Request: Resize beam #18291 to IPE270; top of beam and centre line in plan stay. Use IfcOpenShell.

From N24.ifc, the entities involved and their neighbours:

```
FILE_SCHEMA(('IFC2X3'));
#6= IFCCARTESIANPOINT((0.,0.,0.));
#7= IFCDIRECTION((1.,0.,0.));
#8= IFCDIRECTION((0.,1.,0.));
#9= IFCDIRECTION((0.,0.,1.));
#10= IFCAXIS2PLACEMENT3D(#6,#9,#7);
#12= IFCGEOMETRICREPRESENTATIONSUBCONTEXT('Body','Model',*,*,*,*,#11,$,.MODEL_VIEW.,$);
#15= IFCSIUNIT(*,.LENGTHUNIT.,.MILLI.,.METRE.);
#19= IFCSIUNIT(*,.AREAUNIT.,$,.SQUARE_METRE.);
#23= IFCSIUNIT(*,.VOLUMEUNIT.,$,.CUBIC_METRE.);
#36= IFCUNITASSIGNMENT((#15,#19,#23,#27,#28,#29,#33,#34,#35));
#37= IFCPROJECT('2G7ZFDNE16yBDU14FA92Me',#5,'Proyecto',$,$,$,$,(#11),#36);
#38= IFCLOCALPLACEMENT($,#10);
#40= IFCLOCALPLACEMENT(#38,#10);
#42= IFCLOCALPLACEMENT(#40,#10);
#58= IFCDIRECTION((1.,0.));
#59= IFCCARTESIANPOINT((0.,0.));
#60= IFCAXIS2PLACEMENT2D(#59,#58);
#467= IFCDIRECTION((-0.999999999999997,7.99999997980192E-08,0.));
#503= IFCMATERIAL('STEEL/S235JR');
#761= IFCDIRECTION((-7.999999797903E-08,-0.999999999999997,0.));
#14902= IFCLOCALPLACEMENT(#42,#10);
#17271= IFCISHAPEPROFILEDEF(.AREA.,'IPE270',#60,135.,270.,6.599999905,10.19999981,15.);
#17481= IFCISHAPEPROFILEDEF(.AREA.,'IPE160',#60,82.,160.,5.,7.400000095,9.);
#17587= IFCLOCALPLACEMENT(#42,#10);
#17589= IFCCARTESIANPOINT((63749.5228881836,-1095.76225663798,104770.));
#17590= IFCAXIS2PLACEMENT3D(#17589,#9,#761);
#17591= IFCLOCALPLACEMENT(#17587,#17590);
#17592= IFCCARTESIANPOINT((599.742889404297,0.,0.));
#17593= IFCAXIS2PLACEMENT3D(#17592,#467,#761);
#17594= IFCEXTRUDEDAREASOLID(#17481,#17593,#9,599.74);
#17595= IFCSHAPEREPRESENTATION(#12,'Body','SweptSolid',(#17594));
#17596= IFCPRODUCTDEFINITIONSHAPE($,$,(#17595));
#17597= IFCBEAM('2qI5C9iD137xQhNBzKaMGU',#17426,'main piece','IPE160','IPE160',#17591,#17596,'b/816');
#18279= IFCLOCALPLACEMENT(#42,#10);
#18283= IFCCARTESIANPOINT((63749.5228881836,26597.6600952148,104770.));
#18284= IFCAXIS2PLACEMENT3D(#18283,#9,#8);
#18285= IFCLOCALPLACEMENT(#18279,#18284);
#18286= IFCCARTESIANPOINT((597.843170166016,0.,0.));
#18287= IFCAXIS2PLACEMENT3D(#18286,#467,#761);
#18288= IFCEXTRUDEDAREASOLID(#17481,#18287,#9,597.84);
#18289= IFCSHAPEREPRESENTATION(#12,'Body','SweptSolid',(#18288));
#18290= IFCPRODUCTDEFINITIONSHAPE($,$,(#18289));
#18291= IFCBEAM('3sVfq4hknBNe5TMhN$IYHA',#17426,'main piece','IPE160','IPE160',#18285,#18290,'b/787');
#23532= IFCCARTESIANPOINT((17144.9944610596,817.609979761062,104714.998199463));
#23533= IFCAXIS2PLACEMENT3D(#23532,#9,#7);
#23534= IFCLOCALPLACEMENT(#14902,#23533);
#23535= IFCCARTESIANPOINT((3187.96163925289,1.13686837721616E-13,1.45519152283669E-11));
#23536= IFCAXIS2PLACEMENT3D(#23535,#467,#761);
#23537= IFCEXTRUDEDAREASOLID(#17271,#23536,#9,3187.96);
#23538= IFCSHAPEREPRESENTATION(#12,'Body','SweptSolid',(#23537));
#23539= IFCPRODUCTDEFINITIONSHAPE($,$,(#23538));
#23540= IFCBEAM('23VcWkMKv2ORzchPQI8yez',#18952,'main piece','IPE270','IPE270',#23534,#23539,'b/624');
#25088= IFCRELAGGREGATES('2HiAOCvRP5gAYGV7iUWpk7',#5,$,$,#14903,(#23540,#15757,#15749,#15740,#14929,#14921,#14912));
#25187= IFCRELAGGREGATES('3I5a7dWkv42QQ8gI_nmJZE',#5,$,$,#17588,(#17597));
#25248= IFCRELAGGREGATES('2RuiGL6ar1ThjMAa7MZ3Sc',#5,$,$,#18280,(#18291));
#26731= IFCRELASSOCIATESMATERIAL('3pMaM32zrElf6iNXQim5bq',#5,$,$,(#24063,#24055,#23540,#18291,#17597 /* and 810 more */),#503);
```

```python
import ifcopenshell
import ifcopenshell.util.element
import ifcopenshell.util.representation

model = ifcopenshell.open("N24.ifc")

member = model.by_guid("3sVfq4hknBNe5TMhN$IYHA")
source = next(p for p in model.by_type("IfcIShapeProfileDef") if p.ProfileName == "IPE270")

body = ifcopenshell.util.representation.get_representation(member, "Model", "Body")
solid = body.Items[0]
old_profile = solid.SweptArea

# Copy the section's sizes but keep this member's own profile position.
profile = ifcopenshell.util.element.copy(model, source)
# Profiles are centred, so shift by half the change in depth to hold the top.
shift = (old_profile.OverallDepth - profile.OverallDepth) / 2
x, y = old_profile.Position.Location.Coordinates
up = (0.0, 1.0)  # upwards, in the solid's own plane
location = model.createIfcCartesianPoint((x + up[0] * shift, y + up[1] * shift))
profile.Position = model.createIfcAxis2Placement2D(location, old_profile.Position.RefDirection)
solid.SweptArea = profile
if not model.get_total_inverses(old_profile):
    ifcopenshell.util.element.remove_deep2(model, old_profile)
member.Description = member.Description.replace("IPE160", "IPE270")
member.ObjectType = member.ObjectType.replace("IPE160", "IPE270")

print(solid.SweptArea)

model.write("N24_rev.ifc")
```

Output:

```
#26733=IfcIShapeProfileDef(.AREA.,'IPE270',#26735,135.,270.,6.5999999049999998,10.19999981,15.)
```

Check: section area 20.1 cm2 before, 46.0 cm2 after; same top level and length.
